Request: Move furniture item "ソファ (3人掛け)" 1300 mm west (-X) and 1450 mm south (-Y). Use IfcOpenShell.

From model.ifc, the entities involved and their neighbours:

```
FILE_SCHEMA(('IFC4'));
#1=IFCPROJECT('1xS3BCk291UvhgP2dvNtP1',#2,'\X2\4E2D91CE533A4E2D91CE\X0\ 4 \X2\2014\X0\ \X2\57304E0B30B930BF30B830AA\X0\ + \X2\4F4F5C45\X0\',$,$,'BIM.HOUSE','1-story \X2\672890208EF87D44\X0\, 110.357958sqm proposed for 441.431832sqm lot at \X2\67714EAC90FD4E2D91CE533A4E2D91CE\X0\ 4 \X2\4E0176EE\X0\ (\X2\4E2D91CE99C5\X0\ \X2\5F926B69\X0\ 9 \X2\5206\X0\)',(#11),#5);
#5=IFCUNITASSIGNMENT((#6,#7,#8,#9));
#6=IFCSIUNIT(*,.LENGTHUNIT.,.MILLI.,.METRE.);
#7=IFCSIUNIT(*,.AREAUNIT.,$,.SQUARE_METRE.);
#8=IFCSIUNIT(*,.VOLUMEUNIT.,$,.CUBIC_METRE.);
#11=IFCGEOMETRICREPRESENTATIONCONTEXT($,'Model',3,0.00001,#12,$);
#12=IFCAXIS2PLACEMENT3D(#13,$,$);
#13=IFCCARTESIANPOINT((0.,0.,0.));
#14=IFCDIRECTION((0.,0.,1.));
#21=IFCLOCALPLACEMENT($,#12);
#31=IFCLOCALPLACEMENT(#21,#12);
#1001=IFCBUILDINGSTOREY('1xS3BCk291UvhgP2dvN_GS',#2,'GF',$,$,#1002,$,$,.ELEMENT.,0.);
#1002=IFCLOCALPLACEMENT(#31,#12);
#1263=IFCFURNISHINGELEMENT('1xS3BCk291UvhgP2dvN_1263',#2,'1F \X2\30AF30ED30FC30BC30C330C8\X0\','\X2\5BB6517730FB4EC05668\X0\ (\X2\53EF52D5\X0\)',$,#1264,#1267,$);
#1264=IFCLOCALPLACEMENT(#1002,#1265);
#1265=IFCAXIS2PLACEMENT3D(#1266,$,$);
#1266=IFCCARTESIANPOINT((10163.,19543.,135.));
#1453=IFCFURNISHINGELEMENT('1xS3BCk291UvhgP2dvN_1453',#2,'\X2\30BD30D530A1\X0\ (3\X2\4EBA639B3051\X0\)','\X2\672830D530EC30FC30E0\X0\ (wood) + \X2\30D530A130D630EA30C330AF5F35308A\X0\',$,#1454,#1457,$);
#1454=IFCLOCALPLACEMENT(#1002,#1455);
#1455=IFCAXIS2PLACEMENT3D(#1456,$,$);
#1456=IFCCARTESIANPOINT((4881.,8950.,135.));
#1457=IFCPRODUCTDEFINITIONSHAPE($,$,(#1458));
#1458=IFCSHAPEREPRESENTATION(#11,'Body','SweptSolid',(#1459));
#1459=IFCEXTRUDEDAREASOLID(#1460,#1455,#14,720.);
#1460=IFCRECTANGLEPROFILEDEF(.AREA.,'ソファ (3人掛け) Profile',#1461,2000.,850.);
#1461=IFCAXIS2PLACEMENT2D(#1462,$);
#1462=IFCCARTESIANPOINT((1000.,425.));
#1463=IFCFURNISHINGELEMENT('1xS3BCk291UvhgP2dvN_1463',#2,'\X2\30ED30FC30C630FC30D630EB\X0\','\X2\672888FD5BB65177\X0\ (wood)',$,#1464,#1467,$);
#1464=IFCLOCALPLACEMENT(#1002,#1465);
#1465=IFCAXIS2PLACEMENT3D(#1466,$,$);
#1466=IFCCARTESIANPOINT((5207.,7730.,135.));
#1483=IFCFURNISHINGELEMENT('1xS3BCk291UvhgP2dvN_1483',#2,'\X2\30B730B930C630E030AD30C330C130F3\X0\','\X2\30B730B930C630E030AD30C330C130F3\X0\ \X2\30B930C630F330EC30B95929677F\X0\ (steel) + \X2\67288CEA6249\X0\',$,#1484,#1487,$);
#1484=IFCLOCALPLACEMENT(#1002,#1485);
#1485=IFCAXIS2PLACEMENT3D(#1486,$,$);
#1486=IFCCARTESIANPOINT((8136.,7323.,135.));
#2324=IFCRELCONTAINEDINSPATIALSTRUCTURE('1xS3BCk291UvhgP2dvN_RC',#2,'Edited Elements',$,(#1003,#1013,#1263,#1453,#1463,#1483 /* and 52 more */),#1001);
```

```python
import ifcopenshell
import ifcopenshell.api.geometry
import ifcopenshell.util.placement

model = ifcopenshell.open("model.ifc")

item = model.by_guid("1xS3BCk291UvhgP2dvN_1453")
matrix = ifcopenshell.util.placement.get_local_placement(item.ObjectPlacement)
matrix[0, 3] -= 1300.0
matrix[1, 3] -= 1450.0
ifcopenshell.api.geometry.edit_object_placement(model, product=item, matrix=matrix, is_si=False)

print(ifcopenshell.util.placement.get_local_placement(item.ObjectPlacement).round(3) + 0.0)

model.write("model_v2.ifc")
```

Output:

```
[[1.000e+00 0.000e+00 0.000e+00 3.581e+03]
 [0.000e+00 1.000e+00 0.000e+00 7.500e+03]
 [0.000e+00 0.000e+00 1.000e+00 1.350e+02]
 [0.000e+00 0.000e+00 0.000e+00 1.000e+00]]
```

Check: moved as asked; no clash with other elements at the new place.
